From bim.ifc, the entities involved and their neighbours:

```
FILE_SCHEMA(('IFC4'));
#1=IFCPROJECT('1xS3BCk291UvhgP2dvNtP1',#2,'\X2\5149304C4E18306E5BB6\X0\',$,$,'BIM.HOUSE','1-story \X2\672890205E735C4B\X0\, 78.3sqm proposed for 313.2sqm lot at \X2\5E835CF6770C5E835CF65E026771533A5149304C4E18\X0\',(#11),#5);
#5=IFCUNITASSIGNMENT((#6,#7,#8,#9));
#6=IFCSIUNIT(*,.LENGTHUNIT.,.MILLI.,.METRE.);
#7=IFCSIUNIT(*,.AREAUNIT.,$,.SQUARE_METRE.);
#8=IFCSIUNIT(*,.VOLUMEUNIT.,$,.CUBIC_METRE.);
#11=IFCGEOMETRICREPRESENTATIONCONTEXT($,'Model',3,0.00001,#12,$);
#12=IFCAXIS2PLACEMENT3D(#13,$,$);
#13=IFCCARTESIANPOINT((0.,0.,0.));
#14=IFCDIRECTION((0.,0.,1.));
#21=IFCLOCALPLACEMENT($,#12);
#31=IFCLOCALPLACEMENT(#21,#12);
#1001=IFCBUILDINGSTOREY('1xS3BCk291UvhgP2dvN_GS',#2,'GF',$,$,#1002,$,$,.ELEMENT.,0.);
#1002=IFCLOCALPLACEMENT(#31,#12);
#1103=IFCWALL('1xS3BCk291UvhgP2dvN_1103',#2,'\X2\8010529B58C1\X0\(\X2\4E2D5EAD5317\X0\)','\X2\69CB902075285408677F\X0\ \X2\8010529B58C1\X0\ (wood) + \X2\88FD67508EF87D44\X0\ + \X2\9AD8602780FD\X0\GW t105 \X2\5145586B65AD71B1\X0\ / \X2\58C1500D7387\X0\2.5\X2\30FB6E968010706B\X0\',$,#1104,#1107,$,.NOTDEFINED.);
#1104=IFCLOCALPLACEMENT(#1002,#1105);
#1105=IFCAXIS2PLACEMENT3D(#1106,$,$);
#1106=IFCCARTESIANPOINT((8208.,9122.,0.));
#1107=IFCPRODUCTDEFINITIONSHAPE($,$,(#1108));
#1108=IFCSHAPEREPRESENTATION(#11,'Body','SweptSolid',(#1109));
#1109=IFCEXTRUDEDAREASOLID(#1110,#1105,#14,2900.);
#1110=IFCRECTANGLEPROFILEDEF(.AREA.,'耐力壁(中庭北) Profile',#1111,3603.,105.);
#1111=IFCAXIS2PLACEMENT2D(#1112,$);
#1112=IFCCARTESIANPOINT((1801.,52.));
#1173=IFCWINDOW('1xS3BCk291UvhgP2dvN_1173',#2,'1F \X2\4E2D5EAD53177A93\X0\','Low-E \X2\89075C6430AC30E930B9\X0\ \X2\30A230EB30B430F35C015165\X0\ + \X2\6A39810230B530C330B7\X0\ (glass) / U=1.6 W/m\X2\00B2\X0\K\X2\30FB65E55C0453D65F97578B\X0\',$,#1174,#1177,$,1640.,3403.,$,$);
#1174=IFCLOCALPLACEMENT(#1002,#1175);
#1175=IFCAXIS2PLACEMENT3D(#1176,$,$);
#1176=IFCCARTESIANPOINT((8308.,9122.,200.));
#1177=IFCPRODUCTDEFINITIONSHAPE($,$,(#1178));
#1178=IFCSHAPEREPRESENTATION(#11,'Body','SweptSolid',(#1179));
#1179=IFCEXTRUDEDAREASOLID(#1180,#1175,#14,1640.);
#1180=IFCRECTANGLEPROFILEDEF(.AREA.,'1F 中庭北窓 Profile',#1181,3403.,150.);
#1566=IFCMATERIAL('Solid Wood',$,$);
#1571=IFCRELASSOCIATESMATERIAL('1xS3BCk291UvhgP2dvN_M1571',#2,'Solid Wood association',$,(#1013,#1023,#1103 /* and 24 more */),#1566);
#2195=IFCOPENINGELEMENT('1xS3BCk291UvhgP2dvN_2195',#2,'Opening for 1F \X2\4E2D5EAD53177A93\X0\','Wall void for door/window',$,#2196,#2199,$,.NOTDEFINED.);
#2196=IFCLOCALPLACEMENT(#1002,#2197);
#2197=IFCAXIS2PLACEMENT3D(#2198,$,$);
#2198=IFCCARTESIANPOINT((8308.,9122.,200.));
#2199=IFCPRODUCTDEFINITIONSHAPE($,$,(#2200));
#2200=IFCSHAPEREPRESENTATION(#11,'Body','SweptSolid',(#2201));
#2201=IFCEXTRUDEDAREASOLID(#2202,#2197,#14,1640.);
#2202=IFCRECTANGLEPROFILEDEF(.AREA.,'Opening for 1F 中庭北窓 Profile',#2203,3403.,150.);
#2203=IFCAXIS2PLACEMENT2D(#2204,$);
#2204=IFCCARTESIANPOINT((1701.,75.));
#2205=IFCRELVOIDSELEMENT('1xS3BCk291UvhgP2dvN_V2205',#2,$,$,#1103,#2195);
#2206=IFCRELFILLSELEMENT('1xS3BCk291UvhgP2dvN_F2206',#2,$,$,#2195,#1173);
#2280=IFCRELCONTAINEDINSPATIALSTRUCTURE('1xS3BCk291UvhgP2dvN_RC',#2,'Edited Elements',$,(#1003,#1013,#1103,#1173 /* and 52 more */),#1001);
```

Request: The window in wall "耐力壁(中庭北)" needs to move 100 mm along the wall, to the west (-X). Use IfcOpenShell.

```python
import ifcopenshell
import ifcopenshell.api.geometry
import ifcopenshell.util.placement
import ifcopenshell.util.unit

model = ifcopenshell.open("bim.ifc")
unit_scale = ifcopenshell.util.unit.calculate_unit_scale(model)

window = model.by_guid("1xS3BCk291UvhgP2dvN_1173")
opening = window.FillsVoids[0].RelatingOpeningElement
wall = opening.VoidsElements[0].RelatingBuildingElement

wall_matrix = ifcopenshell.util.placement.get_local_placement(wall.ObjectPlacement)
shift = wall_matrix[:3, 0] * -0.1 / unit_scale
before = ifcopenshell.util.placement.get_local_placement(window.ObjectPlacement)[:3, 3].copy()

# The window is not placed relative to its opening, so move both.
for product in (opening, window):
    matrix = ifcopenshell.util.placement.get_local_placement(product.ObjectPlacement)
    matrix[:3, 3] += shift
    ifcopenshell.api.geometry.edit_object_placement(model, product=product, matrix=matrix, is_si=False)

after = ifcopenshell.util.placement.get_local_placement(window.ObjectPlacement)[:3, 3]
print("window moved by", (after - before).round(3) + 0.0)

model.write("bim_edited.ifc")
```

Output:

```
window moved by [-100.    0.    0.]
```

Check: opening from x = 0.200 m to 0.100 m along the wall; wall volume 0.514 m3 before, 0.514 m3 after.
